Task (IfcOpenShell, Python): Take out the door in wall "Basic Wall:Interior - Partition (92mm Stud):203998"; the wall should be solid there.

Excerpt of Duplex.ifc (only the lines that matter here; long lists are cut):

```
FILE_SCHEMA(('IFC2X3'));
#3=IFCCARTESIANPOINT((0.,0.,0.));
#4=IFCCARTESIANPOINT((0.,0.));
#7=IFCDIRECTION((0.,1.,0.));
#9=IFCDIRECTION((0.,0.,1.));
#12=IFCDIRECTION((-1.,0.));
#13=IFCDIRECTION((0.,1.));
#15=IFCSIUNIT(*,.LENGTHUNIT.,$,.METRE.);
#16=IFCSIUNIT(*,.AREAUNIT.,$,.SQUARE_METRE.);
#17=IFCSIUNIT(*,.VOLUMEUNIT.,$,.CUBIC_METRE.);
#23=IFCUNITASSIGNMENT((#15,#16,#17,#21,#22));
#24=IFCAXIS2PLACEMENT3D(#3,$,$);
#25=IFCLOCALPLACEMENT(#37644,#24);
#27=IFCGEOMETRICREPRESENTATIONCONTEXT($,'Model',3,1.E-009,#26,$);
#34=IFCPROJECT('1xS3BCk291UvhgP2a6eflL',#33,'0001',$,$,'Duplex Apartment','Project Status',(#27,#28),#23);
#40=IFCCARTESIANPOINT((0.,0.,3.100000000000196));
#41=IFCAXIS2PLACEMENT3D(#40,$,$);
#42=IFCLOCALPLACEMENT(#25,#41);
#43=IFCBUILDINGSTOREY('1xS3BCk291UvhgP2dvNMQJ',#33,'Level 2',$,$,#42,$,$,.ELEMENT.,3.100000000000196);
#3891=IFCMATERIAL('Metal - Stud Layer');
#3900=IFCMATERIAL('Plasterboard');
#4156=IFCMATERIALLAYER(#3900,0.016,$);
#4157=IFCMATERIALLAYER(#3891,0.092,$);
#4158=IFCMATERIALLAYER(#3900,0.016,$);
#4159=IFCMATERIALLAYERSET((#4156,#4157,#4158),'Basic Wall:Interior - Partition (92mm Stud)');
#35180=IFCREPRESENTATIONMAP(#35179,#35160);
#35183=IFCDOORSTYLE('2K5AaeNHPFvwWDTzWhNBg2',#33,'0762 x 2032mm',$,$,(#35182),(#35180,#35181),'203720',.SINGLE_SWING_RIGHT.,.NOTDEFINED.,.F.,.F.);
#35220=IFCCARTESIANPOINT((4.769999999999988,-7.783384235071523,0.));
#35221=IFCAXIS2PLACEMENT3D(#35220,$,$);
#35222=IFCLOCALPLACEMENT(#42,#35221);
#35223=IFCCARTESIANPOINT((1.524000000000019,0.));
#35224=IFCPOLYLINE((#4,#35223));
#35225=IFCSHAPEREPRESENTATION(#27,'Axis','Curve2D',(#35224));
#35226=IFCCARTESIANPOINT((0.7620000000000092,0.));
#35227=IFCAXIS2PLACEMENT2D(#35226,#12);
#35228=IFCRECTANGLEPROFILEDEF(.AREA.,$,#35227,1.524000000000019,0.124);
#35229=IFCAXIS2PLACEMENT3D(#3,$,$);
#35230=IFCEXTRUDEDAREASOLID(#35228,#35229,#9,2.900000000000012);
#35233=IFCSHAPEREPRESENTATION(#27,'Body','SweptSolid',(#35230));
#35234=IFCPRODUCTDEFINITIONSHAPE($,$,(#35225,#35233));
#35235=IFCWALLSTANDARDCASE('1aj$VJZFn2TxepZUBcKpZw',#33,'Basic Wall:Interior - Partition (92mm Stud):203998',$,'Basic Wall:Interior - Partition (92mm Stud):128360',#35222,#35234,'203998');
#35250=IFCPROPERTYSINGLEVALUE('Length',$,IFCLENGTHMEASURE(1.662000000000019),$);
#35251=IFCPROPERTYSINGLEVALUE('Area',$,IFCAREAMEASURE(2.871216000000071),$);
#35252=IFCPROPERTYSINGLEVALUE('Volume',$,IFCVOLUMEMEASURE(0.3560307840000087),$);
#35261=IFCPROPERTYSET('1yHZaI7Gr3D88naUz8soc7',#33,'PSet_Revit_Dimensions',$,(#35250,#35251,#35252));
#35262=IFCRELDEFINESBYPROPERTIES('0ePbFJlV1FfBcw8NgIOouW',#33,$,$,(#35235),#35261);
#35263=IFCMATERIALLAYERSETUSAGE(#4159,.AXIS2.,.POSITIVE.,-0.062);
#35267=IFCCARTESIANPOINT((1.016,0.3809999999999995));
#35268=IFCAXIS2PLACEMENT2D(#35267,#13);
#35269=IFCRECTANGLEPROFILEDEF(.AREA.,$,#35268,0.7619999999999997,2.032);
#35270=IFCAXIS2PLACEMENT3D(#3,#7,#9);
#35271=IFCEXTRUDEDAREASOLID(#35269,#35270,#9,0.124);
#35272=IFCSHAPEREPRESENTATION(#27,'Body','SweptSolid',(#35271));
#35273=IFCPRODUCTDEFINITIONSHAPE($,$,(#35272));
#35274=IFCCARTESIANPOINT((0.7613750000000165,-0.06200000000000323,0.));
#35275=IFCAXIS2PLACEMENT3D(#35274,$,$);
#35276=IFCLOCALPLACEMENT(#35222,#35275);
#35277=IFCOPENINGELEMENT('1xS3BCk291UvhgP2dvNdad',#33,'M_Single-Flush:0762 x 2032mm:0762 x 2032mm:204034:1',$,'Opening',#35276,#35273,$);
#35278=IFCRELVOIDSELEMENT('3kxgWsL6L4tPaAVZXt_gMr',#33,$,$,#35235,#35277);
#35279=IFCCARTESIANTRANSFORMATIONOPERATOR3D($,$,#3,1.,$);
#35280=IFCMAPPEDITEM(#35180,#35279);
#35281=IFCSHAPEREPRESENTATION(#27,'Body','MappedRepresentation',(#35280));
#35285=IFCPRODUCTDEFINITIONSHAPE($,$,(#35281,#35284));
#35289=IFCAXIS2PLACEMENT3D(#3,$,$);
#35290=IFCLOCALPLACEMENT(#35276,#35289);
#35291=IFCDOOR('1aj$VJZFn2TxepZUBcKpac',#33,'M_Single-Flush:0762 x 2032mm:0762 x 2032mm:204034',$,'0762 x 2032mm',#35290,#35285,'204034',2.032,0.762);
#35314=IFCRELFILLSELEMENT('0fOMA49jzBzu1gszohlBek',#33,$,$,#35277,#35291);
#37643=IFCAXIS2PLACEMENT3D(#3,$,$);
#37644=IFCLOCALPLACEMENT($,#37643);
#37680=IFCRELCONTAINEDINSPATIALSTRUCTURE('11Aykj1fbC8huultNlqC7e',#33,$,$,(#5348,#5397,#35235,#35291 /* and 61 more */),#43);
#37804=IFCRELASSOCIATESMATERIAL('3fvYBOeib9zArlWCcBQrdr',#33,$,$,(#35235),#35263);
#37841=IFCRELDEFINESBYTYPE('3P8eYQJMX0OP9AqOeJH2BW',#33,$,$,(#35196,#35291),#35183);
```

```python
import ifcopenshell
import ifcopenshell.api.feature
import ifcopenshell.api.pset
import ifcopenshell.api.root
import ifcopenshell.geom
import ifcopenshell.util.element
import ifcopenshell.util.shape
import ifcopenshell.util.unit

model = ifcopenshell.open("Duplex.ifc")
area_scale = ifcopenshell.util.unit.calculate_unit_scale(model, "AREAUNIT")
volume_scale = ifcopenshell.util.unit.calculate_unit_scale(model, "VOLUMEUNIT")
settings = ifcopenshell.geom.settings()


def volume(element):
    """Net volume in cubic metres, openings subtracted."""
    shape = ifcopenshell.geom.create_shape(settings, element)
    return ifcopenshell.util.shape.get_volume(shape.geometry)


door = model.by_guid("1aj$VJZFn2TxepZUBcKpac")
opening = door.FillsVoids[0].RelatingOpeningElement
wall = opening.VoidsElements[0].RelatingBuildingElement
before = volume(wall)

ifcopenshell.api.root.remove_product(model, product=door)
ifcopenshell.api.feature.remove_feature(model, feature=opening)

after = volume(wall)
thickness = 0.124  # wall thickness in metres

# Update the wall's stored quantities.
pset = model.by_id(ifcopenshell.util.element.get_pset(wall, "PSet_Revit_Dimensions", should_inherit=False)["id"])
ifcopenshell.api.pset.edit_pset(model, pset=pset, properties={
    "Area": model.create_entity("IfcAreaMeasure", after / thickness / area_scale),
    "Volume": model.create_entity("IfcVolumeMeasure", after / volume_scale),
})

print(f"wall volume {before:.3f} -> {after:.3f} m3")

model.write("Duplex_v2.ifc")
```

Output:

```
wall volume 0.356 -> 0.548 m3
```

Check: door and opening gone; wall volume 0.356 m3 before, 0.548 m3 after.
